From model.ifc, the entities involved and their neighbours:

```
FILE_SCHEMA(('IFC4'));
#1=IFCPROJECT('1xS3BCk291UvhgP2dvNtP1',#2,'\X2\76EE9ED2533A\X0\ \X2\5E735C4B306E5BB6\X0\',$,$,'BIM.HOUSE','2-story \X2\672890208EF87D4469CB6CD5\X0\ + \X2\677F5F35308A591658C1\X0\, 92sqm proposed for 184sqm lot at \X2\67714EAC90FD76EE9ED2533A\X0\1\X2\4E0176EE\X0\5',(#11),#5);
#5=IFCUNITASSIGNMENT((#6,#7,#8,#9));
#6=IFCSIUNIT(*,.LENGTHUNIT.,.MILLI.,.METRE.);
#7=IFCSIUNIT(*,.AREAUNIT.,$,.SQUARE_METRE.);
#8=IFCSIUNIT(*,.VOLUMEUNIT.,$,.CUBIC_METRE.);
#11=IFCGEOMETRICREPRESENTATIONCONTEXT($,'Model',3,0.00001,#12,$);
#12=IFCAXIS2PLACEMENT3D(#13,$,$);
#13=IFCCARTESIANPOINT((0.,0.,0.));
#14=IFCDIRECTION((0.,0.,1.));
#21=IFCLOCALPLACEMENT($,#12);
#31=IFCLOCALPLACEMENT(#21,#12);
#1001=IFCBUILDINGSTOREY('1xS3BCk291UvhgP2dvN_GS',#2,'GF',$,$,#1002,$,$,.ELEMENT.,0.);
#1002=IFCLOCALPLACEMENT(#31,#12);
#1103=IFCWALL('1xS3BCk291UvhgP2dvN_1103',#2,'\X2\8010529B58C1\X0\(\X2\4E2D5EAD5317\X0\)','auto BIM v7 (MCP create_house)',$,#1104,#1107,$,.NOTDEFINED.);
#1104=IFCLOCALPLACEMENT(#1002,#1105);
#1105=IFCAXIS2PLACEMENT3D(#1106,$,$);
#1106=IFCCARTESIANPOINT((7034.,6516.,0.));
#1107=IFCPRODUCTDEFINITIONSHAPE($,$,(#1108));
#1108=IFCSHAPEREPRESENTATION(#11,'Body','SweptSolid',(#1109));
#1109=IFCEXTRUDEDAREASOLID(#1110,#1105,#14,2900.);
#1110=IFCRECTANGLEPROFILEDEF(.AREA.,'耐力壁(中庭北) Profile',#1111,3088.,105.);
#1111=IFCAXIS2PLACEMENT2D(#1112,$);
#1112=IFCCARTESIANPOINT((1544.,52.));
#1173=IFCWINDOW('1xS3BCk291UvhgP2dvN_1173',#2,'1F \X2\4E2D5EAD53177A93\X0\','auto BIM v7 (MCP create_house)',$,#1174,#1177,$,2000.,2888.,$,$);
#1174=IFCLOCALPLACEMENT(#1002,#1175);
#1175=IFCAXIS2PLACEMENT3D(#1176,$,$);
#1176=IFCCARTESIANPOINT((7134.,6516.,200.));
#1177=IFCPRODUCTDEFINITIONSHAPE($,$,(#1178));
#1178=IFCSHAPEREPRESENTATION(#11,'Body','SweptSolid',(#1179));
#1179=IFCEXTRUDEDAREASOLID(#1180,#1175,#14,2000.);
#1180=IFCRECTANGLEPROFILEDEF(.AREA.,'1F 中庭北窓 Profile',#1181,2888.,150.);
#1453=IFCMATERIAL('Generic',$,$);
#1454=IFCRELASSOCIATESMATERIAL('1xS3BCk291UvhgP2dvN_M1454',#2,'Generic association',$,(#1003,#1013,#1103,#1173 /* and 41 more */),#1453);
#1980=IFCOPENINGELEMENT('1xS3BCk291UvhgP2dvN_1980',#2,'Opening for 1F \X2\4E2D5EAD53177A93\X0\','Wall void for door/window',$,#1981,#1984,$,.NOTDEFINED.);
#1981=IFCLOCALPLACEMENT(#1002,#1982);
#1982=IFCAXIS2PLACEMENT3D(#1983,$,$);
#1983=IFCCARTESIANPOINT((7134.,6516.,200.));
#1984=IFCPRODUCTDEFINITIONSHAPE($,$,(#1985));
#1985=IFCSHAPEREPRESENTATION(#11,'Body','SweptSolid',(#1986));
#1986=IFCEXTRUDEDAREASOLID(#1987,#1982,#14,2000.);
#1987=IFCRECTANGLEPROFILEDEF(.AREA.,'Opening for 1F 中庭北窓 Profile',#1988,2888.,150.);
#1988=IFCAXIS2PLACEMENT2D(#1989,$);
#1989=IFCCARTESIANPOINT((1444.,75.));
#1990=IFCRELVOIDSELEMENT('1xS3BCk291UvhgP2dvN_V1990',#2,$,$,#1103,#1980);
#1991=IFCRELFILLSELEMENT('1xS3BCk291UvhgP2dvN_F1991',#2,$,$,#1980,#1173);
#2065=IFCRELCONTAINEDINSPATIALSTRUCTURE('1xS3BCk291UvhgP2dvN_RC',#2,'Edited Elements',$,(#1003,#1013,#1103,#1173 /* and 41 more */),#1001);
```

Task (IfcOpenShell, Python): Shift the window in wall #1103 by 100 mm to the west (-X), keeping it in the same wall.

```python
import ifcopenshell
import ifcopenshell.api.geometry
import ifcopenshell.util.placement

model = ifcopenshell.open("model.ifc")

window = model.by_guid("1xS3BCk291UvhgP2dvN_1173")
opening = window.FillsVoids[0].RelatingOpeningElement
wall = opening.VoidsElements[0].RelatingBuildingElement

wall_matrix = ifcopenshell.util.placement.get_local_placement(wall.ObjectPlacement)
shift = wall_matrix[:3, 0] * -100.0
before = ifcopenshell.util.placement.get_local_placement(window.ObjectPlacement)[:3, 3].copy()

# The window is not placed relative to its opening, so move both.
for product in (opening, window):
    matrix = ifcopenshell.util.placement.get_local_placement(product.ObjectPlacement)
    matrix[:3, 3] += shift
    ifcopenshell.api.geometry.edit_object_placement(model, product=product, matrix=matrix, is_si=False)

after = ifcopenshell.util.placement.get_local_placement(window.ObjectPlacement)[:3, 3]
print("window moved by", (after - before).round(3) + 0.0)

model.write("model_updated.ifc")
```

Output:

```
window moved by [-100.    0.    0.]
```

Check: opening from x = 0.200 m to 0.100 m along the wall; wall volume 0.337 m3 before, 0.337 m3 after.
